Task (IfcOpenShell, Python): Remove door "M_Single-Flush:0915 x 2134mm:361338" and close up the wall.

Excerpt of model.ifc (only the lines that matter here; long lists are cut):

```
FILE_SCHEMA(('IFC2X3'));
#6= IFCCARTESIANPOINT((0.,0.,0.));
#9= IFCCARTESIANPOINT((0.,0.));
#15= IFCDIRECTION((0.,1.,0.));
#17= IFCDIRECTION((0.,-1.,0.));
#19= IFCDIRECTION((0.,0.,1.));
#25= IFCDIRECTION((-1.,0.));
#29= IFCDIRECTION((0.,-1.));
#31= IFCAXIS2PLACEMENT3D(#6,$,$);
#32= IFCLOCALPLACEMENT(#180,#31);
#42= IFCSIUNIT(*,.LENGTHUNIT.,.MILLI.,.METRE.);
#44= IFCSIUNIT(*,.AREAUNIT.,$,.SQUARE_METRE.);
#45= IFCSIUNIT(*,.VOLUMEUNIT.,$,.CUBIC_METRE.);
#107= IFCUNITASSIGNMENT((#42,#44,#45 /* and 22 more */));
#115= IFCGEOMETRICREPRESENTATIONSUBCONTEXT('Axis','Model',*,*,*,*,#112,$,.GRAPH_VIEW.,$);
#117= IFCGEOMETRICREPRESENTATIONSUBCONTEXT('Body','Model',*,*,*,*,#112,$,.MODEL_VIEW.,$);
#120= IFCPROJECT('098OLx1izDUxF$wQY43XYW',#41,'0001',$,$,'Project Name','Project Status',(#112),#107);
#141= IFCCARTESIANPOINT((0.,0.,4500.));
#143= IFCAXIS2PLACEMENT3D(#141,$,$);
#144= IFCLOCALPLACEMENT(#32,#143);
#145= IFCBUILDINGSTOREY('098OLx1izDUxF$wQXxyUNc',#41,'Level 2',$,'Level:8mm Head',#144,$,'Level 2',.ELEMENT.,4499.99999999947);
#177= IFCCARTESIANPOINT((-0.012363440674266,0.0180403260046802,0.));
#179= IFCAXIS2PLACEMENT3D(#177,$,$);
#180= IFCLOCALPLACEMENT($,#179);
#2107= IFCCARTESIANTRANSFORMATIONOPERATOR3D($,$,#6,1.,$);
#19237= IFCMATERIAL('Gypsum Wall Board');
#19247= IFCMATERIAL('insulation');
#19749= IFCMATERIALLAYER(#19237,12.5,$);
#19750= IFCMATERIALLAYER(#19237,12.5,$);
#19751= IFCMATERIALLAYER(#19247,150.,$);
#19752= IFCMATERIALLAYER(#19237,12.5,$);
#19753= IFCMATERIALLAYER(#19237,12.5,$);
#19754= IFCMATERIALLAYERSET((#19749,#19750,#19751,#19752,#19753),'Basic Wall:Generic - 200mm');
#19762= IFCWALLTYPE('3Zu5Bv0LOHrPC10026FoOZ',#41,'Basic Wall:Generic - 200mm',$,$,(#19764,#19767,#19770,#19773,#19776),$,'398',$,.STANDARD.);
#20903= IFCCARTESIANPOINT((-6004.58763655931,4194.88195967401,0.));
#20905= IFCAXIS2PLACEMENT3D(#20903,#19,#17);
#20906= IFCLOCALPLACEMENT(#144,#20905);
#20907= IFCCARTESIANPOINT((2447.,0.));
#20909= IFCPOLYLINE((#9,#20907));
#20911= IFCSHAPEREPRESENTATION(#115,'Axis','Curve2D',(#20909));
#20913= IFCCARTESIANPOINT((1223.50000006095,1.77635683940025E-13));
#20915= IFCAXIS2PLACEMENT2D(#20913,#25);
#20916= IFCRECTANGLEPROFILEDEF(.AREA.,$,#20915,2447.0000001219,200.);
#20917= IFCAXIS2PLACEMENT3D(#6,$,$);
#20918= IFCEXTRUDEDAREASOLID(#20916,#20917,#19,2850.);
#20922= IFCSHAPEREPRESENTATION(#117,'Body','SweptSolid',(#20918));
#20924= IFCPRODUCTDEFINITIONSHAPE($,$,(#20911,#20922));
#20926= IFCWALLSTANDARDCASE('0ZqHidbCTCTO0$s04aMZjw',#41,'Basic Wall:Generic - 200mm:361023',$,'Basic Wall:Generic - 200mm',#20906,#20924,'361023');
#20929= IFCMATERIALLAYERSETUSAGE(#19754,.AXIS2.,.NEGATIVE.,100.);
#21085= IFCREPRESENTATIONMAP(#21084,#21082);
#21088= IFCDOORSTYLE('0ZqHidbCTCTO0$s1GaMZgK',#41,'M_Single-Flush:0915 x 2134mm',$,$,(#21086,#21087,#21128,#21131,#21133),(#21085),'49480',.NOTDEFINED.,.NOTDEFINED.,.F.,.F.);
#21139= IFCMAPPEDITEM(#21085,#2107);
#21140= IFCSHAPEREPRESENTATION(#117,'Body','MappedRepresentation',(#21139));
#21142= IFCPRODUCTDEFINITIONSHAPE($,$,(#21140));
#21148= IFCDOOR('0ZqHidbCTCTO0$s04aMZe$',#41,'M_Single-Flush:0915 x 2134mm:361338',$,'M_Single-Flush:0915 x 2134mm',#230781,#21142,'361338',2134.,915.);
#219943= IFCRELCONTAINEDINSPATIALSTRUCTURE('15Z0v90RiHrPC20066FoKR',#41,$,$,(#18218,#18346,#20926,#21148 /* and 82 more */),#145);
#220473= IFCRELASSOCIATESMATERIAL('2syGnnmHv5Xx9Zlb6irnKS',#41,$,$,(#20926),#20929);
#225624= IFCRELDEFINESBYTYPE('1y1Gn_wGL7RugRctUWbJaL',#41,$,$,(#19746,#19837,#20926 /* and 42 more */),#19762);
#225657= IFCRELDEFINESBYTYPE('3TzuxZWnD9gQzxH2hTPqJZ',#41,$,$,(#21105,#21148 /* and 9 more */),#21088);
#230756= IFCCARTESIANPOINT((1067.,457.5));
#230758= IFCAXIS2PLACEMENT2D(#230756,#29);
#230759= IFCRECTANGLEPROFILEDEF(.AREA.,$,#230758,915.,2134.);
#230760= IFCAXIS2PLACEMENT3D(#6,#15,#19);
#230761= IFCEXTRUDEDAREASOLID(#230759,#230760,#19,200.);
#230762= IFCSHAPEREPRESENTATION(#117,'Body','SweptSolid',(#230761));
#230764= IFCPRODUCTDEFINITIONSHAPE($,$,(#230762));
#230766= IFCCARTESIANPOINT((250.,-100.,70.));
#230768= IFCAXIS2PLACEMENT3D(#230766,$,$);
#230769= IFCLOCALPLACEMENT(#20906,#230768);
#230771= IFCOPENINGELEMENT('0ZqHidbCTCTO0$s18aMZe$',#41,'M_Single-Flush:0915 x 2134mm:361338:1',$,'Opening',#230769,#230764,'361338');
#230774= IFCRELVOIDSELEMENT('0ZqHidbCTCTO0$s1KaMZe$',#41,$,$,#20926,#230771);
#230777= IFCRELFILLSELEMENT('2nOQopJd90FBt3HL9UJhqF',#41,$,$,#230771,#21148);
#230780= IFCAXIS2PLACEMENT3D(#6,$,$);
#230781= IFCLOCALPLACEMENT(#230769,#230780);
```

```python
import ifcopenshell
import ifcopenshell.api.feature
import ifcopenshell.api.root
import ifcopenshell.geom
import ifcopenshell.util.shape

model = ifcopenshell.open("model.ifc")
settings = ifcopenshell.geom.settings()


def volume(element):
    """Net volume in cubic metres, openings subtracted."""
    shape = ifcopenshell.geom.create_shape(settings, element)
    return ifcopenshell.util.shape.get_volume(shape.geometry)


door = model.by_id(21148)
opening = door.FillsVoids[0].RelatingOpeningElement
wall = opening.VoidsElements[0].RelatingBuildingElement
before = volume(wall)

ifcopenshell.api.root.remove_product(model, product=door)
ifcopenshell.api.feature.remove_feature(model, feature=opening)

after = volume(wall)

print(f"wall volume {before:.3f} -> {after:.3f} m3")

model.write("model_updated.ifc")
```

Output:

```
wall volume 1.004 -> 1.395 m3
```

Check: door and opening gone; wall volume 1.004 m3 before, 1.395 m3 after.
